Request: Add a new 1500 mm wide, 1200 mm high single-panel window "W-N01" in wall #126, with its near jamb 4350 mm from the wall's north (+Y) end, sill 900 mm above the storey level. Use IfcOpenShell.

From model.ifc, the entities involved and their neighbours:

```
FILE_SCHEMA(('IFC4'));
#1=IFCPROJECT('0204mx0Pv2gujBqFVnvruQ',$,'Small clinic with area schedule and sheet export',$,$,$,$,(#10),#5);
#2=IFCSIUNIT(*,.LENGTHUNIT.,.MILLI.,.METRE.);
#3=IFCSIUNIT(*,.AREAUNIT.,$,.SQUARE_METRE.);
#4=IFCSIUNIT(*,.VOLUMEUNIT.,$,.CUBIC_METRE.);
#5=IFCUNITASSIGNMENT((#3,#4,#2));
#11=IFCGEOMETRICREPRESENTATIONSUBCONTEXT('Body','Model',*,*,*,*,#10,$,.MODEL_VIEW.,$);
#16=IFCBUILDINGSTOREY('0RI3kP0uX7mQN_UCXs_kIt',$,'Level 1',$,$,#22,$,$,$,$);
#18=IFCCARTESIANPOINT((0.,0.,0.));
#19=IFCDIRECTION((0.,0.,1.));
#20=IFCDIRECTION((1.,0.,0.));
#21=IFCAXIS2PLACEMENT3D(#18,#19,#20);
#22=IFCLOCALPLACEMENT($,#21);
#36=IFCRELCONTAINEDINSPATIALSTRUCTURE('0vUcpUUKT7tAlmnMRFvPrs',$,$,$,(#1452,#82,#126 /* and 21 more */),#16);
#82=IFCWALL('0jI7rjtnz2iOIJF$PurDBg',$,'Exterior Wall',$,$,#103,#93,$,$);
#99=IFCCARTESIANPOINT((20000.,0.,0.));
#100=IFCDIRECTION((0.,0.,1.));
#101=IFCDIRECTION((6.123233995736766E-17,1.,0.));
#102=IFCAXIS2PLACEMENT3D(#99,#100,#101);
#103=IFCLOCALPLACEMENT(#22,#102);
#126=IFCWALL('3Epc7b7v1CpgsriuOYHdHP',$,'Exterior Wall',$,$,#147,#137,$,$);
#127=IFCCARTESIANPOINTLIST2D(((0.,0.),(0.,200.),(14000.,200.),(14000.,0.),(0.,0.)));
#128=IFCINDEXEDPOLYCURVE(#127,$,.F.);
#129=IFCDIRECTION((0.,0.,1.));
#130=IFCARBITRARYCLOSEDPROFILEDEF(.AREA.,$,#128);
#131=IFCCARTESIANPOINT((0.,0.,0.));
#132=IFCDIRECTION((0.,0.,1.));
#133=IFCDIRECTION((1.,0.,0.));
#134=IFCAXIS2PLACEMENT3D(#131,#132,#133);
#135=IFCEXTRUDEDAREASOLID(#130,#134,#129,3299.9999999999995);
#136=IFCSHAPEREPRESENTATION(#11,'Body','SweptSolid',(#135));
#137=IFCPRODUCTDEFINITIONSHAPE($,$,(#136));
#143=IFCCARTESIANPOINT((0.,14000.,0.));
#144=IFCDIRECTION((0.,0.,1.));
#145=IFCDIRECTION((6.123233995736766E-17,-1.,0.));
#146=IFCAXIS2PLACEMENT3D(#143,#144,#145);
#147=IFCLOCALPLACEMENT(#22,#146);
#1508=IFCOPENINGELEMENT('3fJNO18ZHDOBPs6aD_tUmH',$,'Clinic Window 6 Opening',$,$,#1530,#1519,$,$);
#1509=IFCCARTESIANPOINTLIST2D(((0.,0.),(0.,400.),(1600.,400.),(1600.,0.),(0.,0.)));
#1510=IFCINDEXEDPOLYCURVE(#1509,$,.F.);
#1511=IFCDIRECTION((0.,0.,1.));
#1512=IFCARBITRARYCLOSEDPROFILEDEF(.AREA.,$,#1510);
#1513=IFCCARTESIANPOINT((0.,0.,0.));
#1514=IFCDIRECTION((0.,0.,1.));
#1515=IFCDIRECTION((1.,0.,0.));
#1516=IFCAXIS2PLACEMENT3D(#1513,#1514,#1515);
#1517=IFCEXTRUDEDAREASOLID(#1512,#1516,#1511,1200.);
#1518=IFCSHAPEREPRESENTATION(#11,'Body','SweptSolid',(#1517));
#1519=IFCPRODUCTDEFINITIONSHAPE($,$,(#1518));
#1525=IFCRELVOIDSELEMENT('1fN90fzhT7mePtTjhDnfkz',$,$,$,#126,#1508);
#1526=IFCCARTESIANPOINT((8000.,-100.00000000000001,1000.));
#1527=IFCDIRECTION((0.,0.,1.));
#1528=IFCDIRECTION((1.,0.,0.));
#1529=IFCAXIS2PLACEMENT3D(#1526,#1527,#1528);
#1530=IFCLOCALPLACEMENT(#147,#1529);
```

```python
import numpy as np
import ifcopenshell
import ifcopenshell.api.feature
import ifcopenshell.api.geometry
import ifcopenshell.api.root
import ifcopenshell.api.spatial
import ifcopenshell.geom
import ifcopenshell.util.element
import ifcopenshell.util.placement
import ifcopenshell.util.representation
import ifcopenshell.util.shape
import ifcopenshell.util.unit

model = ifcopenshell.open("model.ifc")
unit_scale = ifcopenshell.util.unit.calculate_unit_scale(model)
settings = ifcopenshell.geom.settings()


def volume(element):
    """Net volume in cubic metres, openings subtracted."""
    shape = ifcopenshell.geom.create_shape(settings, element)
    return ifcopenshell.util.shape.get_volume(shape.geometry)


wall = model.by_id(126)
storey = ifcopenshell.util.element.get_container(wall, ifc_class="IfcBuildingStorey")
context = ifcopenshell.util.representation.get_context(model, "Model", "Body", "MODEL_VIEW")
before = volume(wall)

width, height, from_end, sill = 1.5, 1.2, 4.35, 0.9  # metres

# The wall runs along its own X axis, and the end named is its -X end.
wall_shape = ifcopenshell.geom.create_shape(settings, wall)
x, y, z = ifcopenshell.util.shape.get_vertices(wall_shape.geometry).T
start = x.min() + from_end
face, thickness = float(y.min()), float(y.max() - y.min())
wall_matrix = ifcopenshell.util.placement.get_local_placement(wall.ObjectPlacement)
level = ifcopenshell.util.placement.get_local_placement(storey.ObjectPlacement)[2, 3]


def in_wall(x, y):
    """Placement at x, y metres in the wall's axes, at sill height."""
    matrix = wall_matrix.copy()
    matrix[:, 3] = wall_matrix @ np.array([x / unit_scale, y / unit_scale, 0.0, 1.0])
    matrix[2, 3] = level + sill / unit_scale
    return matrix


# Opening: a box that overshoots both wall faces by 50 mm.
opening = ifcopenshell.api.root.create_entity(model, ifc_class="IfcOpeningElement", predefined_type="OPENING")
box = ifcopenshell.api.geometry.add_wall_representation(
    model, context=context, length=width, height=height, thickness=thickness + 0.1
)
ifcopenshell.api.geometry.assign_representation(model, product=opening, representation=box)
ifcopenshell.api.geometry.edit_object_placement(model, product=opening, matrix=in_wall(start, face - 0.05), is_si=False)
ifcopenshell.api.feature.add_feature(model, feature=opening, element=wall)

window = ifcopenshell.api.root.create_entity(model, ifc_class="IfcWindow", name="W-N01", predefined_type="WINDOW")
window.OverallWidth, window.OverallHeight = width / unit_scale, height / unit_scale
window.PartitioningType = "SINGLE_PANEL"
body = ifcopenshell.api.geometry.add_window_representation(
    model,
    context=context,
    overall_width=window.OverallWidth,
    overall_height=window.OverallHeight,
    partition_type="SINGLE_PANEL",
)
ifcopenshell.api.geometry.assign_representation(model, product=window, representation=body)
ifcopenshell.api.spatial.assign_container(model, products=[window], relating_structure=storey)
ifcopenshell.api.feature.add_filling(model, opening=opening, element=window)

# Centre the window in the wall's thickness.
ifcopenshell.api.geometry.edit_object_placement(model, product=window, matrix=in_wall(start, face), is_si=False)
window_shape = ifcopenshell.geom.create_shape(settings, window)
depth = ifcopenshell.util.shape.get_vertices(window_shape.geometry)[:, 1]
offset = face + thickness / 2 - (depth.min() + depth.max()) / 2
ifcopenshell.api.geometry.edit_object_placement(model, product=window, matrix=in_wall(start, offset), is_si=False)

after = volume(wall)

print(f"wall volume {before:.3f} -> {after:.3f} m3")

model.write("model-out.ifc")
```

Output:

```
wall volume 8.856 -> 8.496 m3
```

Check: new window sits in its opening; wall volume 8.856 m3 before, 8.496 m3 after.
